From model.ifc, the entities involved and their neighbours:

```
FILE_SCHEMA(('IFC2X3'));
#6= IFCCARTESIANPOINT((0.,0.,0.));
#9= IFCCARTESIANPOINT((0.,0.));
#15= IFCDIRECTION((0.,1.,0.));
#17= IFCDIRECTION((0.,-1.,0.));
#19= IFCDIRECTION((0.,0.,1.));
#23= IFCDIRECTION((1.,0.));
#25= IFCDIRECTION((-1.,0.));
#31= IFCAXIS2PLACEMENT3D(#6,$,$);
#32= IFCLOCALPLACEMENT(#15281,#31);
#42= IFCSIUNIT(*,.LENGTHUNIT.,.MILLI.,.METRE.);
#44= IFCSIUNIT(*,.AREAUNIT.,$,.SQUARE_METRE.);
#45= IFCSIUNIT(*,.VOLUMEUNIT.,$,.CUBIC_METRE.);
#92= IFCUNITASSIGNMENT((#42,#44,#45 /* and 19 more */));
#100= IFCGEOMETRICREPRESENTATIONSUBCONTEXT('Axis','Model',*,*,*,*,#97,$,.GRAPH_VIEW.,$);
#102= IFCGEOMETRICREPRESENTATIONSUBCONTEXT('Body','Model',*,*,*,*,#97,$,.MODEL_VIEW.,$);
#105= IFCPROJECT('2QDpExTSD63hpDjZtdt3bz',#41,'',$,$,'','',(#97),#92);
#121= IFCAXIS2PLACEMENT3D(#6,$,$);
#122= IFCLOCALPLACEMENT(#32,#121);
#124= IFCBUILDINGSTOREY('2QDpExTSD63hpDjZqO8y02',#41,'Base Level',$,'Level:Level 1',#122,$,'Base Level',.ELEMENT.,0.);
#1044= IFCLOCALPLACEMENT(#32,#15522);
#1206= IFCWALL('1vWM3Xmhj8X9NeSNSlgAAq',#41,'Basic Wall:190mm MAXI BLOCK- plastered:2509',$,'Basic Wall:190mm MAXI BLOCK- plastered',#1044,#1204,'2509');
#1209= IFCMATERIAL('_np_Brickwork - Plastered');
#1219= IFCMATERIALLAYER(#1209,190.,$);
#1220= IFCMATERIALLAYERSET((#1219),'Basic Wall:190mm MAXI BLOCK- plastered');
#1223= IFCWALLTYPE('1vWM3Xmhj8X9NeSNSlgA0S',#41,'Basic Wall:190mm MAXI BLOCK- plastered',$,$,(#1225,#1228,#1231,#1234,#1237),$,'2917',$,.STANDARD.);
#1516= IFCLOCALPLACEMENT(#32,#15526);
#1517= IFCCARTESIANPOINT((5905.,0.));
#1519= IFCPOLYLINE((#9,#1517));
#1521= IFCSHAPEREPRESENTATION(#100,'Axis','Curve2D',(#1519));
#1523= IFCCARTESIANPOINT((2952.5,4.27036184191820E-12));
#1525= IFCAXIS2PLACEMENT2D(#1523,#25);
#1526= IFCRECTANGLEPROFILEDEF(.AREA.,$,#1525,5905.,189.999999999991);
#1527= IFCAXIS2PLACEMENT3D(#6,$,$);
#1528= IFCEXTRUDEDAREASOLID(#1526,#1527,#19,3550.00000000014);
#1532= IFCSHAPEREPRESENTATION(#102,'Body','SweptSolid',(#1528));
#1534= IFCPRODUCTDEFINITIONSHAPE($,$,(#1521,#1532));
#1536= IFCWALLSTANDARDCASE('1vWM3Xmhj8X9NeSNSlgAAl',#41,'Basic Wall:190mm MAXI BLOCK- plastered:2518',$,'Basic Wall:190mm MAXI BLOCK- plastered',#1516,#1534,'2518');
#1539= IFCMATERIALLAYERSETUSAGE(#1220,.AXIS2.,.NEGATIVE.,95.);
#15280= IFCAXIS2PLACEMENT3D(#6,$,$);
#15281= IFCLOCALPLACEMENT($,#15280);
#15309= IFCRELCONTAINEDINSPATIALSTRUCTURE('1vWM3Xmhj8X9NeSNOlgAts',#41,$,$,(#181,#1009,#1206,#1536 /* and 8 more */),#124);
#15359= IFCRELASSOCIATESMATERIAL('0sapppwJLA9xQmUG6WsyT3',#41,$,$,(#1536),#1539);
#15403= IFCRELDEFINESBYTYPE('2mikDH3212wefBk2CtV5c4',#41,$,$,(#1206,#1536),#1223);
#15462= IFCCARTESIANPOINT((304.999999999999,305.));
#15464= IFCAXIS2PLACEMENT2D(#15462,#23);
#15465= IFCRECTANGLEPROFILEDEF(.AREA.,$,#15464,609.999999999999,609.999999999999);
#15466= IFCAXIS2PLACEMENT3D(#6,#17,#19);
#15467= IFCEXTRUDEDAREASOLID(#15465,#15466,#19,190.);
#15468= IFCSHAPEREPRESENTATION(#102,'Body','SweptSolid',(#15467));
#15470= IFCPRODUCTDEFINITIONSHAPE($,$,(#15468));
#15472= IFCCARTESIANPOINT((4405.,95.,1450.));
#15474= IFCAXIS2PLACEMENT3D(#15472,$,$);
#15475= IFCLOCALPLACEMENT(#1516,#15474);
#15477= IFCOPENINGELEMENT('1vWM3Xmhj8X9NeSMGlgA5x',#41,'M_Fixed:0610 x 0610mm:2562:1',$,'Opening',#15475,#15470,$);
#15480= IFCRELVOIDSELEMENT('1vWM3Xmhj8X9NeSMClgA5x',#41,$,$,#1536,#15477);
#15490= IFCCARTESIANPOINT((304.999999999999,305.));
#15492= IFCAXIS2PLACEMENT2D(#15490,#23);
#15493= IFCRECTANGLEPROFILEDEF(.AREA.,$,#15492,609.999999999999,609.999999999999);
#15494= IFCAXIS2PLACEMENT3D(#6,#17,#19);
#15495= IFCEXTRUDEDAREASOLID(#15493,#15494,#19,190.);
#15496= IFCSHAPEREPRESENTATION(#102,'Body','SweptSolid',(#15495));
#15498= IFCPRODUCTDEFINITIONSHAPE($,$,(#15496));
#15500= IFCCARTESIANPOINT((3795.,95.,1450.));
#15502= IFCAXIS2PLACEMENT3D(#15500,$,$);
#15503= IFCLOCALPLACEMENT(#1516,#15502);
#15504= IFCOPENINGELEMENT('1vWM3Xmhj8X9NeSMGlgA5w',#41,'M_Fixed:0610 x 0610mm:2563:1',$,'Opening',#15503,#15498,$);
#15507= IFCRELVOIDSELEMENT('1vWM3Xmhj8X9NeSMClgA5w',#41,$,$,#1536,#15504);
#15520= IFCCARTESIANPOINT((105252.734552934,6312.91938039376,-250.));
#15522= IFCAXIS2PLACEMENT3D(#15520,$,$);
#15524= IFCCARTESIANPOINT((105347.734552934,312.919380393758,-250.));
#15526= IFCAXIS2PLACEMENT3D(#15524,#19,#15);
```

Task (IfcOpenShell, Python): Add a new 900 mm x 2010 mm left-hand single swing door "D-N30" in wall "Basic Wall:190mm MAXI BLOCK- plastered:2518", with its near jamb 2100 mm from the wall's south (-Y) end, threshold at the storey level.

```python
import numpy as np
import ifcopenshell
import ifcopenshell.api.feature
import ifcopenshell.api.geometry
import ifcopenshell.api.root
import ifcopenshell.api.spatial
import ifcopenshell.api.type
import ifcopenshell.geom
import ifcopenshell.util.element
import ifcopenshell.util.placement
import ifcopenshell.util.representation
import ifcopenshell.util.shape
import ifcopenshell.util.unit

model = ifcopenshell.open("model.ifc")
unit_scale = ifcopenshell.util.unit.calculate_unit_scale(model)
settings = ifcopenshell.geom.settings()


def volume(element):
    """Net volume in cubic metres, openings subtracted."""
    shape = ifcopenshell.geom.create_shape(settings, element)
    return ifcopenshell.util.shape.get_volume(shape.geometry)


wall = model.by_id(1536)
storey = ifcopenshell.util.element.get_container(wall, ifc_class="IfcBuildingStorey")
context = ifcopenshell.util.representation.get_context(model, "Model", "Body", "MODEL_VIEW")
before = volume(wall)

width, height, from_end, sill = 0.9, 2.01, 2.1, 0.0  # metres

# The wall runs along its own X axis, and the end named is its -X end.
wall_shape = ifcopenshell.geom.create_shape(settings, wall)
x, y, z = ifcopenshell.util.shape.get_vertices(wall_shape.geometry).T
start = x.min() + from_end
face, thickness = float(y.min()), float(y.max() - y.min())
wall_matrix = ifcopenshell.util.placement.get_local_placement(wall.ObjectPlacement)
level = ifcopenshell.util.placement.get_local_placement(storey.ObjectPlacement)[2, 3]


def in_wall(x, y):
    """Placement at x, y metres in the wall's axes, at sill height."""
    matrix = wall_matrix.copy()
    matrix[:, 3] = wall_matrix @ np.array([x / unit_scale, y / unit_scale, 0.0, 1.0])
    matrix[2, 3] = level + sill / unit_scale
    return matrix


# Opening: a box that overshoots both wall faces by 50 mm.
opening = ifcopenshell.api.root.create_entity(model, ifc_class="IfcOpeningElement")
box = ifcopenshell.api.geometry.add_wall_representation(
    model, context=context, length=width, height=height, thickness=thickness + 0.1
)
ifcopenshell.api.geometry.assign_representation(model, product=opening, representation=box)
ifcopenshell.api.geometry.edit_object_placement(model, product=opening, matrix=in_wall(start, face - 0.05), is_si=False)
ifcopenshell.api.feature.add_feature(model, feature=opening, element=wall)

door = ifcopenshell.api.root.create_entity(model, ifc_class="IfcDoor", name="D-N30")
door.OverallWidth, door.OverallHeight = width / unit_scale, height / unit_scale
body = ifcopenshell.api.geometry.add_door_representation(
    model,
    context=context,
    overall_width=door.OverallWidth,
    overall_height=door.OverallHeight,
    operation_type="SINGLE_SWING_LEFT",
    lining_properties={"LiningDepth": thickness / unit_scale, "ThresholdDepth": thickness / unit_scale},
)
ifcopenshell.api.geometry.assign_representation(model, product=door, representation=body)
ifcopenshell.api.spatial.assign_container(model, products=[door], relating_structure=storey)
fills = ifcopenshell.api.feature.add_filling(model, opening=opening, element=door)
fills.OwnerHistory = door.OwnerHistory  # required in IFC2X3

# IFC2X3 keeps the operation on the door style.
style = ifcopenshell.api.root.create_entity(model, ifc_class="IfcDoorStyle", name="D-N30")
style.OperationType, style.ConstructionType = "SINGLE_SWING_LEFT", "NOTDEFINED"
style.ParameterTakesPrecedence = style.Sizeable = False
ifcopenshell.api.type.assign_type(model, related_objects=[door], relating_type=style)

# The lining spans the wall, so the door starts at the wall face.
ifcopenshell.api.geometry.edit_object_placement(model, product=door, matrix=in_wall(start, face), is_si=False)

after = volume(wall)

print(f"wall volume {before:.3f} -> {after:.3f} m3")

model.write("model-out.ifc")
```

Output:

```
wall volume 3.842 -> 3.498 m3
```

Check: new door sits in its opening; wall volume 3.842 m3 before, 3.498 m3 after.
